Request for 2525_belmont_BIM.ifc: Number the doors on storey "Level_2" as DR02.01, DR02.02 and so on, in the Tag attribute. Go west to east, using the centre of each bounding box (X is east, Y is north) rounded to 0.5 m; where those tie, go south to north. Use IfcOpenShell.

First a look at what the model holds.

```python
import ifcopenshell
import ifcopenshell.util.element
import ifcopenshell.util.placement

model = ifcopenshell.open("2525_belmont_BIM.ifc")
print(model.schema)
storey = next(s for s in model.by_type("IfcBuildingStorey") if s.Name == "Level_2")
doors = [e for e in ifcopenshell.util.element.get_decomposition(storey) if e.is_a("IfcDoor")]
for e in sorted(doors, key=lambda e: e.id()):
    origin = ifcopenshell.util.placement.get_local_placement(e.ObjectPlacement)[:3, 3]
    print(e.id(), e.Tag, e.Name, origin.round(2) + 0.0, sep=" | ")
```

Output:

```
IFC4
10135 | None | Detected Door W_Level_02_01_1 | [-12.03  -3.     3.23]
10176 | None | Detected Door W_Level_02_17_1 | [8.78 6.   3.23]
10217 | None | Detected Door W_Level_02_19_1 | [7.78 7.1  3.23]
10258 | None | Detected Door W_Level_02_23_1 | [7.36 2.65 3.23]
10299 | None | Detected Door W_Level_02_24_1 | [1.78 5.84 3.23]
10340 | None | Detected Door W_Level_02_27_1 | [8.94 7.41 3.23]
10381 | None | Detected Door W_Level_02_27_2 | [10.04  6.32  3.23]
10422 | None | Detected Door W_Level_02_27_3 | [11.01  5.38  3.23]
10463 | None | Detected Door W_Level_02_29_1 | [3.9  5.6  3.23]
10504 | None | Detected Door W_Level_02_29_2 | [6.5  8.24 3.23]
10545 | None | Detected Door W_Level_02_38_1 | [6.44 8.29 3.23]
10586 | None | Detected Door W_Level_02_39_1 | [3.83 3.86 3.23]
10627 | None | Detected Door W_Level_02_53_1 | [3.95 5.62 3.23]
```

```python
import ifcopenshell
import ifcopenshell.geom
import ifcopenshell.util.element
import ifcopenshell.util.shape

model = ifcopenshell.open("2525_belmont_BIM.ifc")
settings = ifcopenshell.geom.settings()
settings.set("use-world-coords", True)


def centre(element):
    shape = ifcopenshell.geom.create_shape(settings, element)
    return ifcopenshell.util.shape.get_bbox_centroid(shape.geometry)


storey = next(s for s in model.by_type("IfcBuildingStorey") if s.Name == "Level_2")
doors = [e for e in ifcopenshell.util.element.get_decomposition(storey) if e.is_a("IfcDoor")]

# Insertion points can sit at a corner or the storey origin, so sort by the geometry (in metres).
centres = {e: centre(e) for e in doors}
doors.sort(key=lambda e: (round(centres[e][0] / 0.5), centres[e][1]))

for i, e in enumerate(doors, start=1):
    number = f"DR02.{i:02d}"
    e.Tag = number
    print(e.id(), number)

model.write("2525_belmont_BIM_updated.ifc")
```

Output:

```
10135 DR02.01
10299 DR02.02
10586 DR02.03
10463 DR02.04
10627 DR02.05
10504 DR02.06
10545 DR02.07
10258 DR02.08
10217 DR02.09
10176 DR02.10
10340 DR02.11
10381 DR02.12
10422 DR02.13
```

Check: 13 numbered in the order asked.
